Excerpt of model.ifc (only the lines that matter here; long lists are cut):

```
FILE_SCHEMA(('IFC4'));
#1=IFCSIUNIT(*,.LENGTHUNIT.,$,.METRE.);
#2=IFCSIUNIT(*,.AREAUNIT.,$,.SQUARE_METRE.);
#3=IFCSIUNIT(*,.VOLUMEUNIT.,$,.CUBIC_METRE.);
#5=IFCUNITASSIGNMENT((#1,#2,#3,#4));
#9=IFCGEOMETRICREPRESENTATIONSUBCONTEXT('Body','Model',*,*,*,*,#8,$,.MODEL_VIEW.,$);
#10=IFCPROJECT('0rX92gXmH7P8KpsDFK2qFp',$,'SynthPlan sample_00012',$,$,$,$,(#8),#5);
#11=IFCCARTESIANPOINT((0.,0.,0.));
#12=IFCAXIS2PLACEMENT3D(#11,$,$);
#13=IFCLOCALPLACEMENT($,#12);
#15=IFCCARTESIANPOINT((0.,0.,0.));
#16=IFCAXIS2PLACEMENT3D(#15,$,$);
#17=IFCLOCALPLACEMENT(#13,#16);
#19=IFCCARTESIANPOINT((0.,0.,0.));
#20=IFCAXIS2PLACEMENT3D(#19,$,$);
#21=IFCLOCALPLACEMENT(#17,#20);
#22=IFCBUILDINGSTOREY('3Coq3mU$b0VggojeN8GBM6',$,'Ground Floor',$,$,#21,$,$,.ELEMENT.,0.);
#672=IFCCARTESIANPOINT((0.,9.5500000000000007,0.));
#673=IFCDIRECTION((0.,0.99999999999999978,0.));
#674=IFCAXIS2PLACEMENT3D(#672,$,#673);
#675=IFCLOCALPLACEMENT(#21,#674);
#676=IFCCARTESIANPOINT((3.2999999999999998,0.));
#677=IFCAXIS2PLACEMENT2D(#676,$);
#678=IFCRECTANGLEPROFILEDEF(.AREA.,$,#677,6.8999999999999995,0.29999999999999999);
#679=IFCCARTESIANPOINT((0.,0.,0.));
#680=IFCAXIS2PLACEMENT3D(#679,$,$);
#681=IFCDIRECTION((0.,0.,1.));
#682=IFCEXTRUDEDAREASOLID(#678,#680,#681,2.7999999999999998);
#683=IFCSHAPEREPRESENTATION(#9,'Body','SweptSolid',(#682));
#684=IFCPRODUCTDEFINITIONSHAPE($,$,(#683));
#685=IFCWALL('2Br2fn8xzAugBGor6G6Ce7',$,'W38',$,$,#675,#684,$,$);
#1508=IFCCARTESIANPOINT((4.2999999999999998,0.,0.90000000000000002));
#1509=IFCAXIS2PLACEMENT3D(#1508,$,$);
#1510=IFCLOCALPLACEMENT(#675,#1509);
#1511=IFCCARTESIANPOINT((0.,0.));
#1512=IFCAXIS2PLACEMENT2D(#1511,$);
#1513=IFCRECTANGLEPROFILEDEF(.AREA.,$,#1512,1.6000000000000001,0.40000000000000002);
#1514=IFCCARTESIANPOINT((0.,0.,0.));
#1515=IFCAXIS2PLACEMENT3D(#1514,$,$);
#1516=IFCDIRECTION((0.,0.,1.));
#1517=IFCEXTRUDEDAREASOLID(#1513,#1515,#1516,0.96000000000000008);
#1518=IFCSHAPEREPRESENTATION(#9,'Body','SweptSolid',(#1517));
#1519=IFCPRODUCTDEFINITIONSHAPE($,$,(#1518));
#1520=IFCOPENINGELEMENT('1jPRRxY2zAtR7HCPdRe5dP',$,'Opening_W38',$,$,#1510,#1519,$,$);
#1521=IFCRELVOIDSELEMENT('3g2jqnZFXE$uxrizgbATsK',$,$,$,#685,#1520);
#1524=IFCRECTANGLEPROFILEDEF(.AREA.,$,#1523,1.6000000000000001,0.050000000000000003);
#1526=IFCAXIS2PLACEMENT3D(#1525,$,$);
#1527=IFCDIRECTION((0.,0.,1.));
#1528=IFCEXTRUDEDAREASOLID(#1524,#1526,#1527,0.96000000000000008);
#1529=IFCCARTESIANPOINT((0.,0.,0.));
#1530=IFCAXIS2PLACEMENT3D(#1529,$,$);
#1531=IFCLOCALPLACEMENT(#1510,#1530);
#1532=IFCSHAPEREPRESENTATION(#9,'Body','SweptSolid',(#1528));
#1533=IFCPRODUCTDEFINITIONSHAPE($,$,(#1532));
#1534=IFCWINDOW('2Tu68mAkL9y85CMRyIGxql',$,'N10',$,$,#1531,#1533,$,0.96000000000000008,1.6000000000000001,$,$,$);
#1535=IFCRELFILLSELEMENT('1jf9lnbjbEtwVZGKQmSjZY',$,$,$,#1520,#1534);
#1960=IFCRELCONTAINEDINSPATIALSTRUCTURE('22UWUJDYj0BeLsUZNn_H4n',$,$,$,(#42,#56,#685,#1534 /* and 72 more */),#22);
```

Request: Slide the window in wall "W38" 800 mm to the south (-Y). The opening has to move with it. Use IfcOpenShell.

```python
import ifcopenshell
import ifcopenshell.api.geometry
import ifcopenshell.util.placement
import ifcopenshell.util.unit

model = ifcopenshell.open("model.ifc")
unit_scale = ifcopenshell.util.unit.calculate_unit_scale(model)

window = model.by_guid("2Tu68mAkL9y85CMRyIGxql")
opening = window.FillsVoids[0].RelatingOpeningElement
wall = opening.VoidsElements[0].RelatingBuildingElement

wall_matrix = ifcopenshell.util.placement.get_local_placement(wall.ObjectPlacement)
shift = wall_matrix[:3, 0] * -0.8 / unit_scale
before = ifcopenshell.util.placement.get_local_placement(window.ObjectPlacement)[:3, 3].copy()

# The window is placed relative to its opening, so it follows when the opening moves.
matrix = ifcopenshell.util.placement.get_local_placement(opening.ObjectPlacement)
matrix[:3, 3] += shift
ifcopenshell.api.geometry.edit_object_placement(
    model, product=opening, matrix=matrix, is_si=False, should_transform_children=True
)

after = ifcopenshell.util.placement.get_local_placement(window.ObjectPlacement)[:3, 3]
print("window moved by", (after - before).round(3) + 0.0)

model.write("model-out.ifc")
```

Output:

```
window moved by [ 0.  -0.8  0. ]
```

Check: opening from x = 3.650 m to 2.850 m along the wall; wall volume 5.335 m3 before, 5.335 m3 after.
